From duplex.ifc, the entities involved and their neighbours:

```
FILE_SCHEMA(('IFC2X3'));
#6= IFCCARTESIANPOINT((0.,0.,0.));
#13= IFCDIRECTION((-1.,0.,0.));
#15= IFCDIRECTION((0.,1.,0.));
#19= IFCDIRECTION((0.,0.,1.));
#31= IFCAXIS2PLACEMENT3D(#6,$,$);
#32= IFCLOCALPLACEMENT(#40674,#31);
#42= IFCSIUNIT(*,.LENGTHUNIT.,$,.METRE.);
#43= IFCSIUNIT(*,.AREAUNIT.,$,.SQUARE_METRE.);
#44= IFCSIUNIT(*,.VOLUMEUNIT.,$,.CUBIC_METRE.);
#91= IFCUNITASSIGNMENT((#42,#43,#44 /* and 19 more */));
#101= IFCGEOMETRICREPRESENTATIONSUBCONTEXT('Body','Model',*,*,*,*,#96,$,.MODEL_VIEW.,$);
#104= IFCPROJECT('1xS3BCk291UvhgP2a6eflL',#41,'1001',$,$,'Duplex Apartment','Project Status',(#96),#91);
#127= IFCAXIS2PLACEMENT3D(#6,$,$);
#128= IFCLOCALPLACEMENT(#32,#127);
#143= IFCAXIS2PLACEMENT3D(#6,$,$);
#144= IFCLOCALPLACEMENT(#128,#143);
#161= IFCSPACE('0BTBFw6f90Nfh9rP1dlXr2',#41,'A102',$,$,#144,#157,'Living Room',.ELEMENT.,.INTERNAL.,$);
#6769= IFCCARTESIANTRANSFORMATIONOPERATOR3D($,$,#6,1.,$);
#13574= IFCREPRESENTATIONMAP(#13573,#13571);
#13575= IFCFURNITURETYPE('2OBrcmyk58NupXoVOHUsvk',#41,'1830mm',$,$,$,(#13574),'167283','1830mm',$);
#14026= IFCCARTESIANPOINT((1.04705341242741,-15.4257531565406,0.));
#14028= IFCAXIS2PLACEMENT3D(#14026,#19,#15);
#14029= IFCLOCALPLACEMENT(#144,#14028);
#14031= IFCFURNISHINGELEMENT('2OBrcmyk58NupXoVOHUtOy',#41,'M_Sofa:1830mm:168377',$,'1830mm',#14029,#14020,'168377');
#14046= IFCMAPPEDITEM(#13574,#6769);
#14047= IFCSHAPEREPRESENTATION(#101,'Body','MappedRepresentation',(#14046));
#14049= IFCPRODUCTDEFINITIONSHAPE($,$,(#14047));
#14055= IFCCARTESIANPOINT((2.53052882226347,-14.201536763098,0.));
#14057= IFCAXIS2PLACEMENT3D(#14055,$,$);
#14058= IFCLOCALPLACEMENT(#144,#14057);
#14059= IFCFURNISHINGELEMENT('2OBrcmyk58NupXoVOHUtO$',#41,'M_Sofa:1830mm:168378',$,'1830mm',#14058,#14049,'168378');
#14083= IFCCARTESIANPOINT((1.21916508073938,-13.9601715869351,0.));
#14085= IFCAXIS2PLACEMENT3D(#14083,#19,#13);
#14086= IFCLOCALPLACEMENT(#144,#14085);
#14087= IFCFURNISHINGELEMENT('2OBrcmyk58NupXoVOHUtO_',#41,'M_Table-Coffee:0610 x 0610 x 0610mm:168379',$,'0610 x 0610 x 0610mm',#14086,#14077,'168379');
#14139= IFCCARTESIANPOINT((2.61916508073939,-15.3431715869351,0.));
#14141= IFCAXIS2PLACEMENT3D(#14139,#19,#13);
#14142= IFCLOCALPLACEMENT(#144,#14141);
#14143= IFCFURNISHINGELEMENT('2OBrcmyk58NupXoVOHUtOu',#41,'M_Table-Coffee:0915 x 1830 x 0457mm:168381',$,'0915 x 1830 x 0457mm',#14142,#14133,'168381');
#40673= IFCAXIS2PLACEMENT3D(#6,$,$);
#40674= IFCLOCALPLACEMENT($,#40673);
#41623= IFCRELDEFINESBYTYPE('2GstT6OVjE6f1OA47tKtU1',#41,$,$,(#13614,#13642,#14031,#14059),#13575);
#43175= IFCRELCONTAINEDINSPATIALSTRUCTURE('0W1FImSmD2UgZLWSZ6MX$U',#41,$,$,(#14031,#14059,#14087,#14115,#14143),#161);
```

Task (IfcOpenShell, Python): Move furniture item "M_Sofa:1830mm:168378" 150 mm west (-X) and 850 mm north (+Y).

```python
import ifcopenshell
import ifcopenshell.api.geometry
import ifcopenshell.util.placement
import ifcopenshell.util.unit

model = ifcopenshell.open("duplex.ifc")
unit_scale = ifcopenshell.util.unit.calculate_unit_scale(model)

item = model.by_id(14059)
matrix = ifcopenshell.util.placement.get_local_placement(item.ObjectPlacement)
matrix[0, 3] -= 0.15 / unit_scale
matrix[1, 3] += 0.85 / unit_scale
ifcopenshell.api.geometry.edit_object_placement(model, product=item, matrix=matrix, is_si=False)

print(ifcopenshell.util.placement.get_local_placement(item.ObjectPlacement).round(3) + 0.0)

model.write("duplex_v2.ifc")
```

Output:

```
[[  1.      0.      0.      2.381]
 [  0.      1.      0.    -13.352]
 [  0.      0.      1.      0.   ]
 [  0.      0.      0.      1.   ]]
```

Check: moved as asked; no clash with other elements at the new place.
